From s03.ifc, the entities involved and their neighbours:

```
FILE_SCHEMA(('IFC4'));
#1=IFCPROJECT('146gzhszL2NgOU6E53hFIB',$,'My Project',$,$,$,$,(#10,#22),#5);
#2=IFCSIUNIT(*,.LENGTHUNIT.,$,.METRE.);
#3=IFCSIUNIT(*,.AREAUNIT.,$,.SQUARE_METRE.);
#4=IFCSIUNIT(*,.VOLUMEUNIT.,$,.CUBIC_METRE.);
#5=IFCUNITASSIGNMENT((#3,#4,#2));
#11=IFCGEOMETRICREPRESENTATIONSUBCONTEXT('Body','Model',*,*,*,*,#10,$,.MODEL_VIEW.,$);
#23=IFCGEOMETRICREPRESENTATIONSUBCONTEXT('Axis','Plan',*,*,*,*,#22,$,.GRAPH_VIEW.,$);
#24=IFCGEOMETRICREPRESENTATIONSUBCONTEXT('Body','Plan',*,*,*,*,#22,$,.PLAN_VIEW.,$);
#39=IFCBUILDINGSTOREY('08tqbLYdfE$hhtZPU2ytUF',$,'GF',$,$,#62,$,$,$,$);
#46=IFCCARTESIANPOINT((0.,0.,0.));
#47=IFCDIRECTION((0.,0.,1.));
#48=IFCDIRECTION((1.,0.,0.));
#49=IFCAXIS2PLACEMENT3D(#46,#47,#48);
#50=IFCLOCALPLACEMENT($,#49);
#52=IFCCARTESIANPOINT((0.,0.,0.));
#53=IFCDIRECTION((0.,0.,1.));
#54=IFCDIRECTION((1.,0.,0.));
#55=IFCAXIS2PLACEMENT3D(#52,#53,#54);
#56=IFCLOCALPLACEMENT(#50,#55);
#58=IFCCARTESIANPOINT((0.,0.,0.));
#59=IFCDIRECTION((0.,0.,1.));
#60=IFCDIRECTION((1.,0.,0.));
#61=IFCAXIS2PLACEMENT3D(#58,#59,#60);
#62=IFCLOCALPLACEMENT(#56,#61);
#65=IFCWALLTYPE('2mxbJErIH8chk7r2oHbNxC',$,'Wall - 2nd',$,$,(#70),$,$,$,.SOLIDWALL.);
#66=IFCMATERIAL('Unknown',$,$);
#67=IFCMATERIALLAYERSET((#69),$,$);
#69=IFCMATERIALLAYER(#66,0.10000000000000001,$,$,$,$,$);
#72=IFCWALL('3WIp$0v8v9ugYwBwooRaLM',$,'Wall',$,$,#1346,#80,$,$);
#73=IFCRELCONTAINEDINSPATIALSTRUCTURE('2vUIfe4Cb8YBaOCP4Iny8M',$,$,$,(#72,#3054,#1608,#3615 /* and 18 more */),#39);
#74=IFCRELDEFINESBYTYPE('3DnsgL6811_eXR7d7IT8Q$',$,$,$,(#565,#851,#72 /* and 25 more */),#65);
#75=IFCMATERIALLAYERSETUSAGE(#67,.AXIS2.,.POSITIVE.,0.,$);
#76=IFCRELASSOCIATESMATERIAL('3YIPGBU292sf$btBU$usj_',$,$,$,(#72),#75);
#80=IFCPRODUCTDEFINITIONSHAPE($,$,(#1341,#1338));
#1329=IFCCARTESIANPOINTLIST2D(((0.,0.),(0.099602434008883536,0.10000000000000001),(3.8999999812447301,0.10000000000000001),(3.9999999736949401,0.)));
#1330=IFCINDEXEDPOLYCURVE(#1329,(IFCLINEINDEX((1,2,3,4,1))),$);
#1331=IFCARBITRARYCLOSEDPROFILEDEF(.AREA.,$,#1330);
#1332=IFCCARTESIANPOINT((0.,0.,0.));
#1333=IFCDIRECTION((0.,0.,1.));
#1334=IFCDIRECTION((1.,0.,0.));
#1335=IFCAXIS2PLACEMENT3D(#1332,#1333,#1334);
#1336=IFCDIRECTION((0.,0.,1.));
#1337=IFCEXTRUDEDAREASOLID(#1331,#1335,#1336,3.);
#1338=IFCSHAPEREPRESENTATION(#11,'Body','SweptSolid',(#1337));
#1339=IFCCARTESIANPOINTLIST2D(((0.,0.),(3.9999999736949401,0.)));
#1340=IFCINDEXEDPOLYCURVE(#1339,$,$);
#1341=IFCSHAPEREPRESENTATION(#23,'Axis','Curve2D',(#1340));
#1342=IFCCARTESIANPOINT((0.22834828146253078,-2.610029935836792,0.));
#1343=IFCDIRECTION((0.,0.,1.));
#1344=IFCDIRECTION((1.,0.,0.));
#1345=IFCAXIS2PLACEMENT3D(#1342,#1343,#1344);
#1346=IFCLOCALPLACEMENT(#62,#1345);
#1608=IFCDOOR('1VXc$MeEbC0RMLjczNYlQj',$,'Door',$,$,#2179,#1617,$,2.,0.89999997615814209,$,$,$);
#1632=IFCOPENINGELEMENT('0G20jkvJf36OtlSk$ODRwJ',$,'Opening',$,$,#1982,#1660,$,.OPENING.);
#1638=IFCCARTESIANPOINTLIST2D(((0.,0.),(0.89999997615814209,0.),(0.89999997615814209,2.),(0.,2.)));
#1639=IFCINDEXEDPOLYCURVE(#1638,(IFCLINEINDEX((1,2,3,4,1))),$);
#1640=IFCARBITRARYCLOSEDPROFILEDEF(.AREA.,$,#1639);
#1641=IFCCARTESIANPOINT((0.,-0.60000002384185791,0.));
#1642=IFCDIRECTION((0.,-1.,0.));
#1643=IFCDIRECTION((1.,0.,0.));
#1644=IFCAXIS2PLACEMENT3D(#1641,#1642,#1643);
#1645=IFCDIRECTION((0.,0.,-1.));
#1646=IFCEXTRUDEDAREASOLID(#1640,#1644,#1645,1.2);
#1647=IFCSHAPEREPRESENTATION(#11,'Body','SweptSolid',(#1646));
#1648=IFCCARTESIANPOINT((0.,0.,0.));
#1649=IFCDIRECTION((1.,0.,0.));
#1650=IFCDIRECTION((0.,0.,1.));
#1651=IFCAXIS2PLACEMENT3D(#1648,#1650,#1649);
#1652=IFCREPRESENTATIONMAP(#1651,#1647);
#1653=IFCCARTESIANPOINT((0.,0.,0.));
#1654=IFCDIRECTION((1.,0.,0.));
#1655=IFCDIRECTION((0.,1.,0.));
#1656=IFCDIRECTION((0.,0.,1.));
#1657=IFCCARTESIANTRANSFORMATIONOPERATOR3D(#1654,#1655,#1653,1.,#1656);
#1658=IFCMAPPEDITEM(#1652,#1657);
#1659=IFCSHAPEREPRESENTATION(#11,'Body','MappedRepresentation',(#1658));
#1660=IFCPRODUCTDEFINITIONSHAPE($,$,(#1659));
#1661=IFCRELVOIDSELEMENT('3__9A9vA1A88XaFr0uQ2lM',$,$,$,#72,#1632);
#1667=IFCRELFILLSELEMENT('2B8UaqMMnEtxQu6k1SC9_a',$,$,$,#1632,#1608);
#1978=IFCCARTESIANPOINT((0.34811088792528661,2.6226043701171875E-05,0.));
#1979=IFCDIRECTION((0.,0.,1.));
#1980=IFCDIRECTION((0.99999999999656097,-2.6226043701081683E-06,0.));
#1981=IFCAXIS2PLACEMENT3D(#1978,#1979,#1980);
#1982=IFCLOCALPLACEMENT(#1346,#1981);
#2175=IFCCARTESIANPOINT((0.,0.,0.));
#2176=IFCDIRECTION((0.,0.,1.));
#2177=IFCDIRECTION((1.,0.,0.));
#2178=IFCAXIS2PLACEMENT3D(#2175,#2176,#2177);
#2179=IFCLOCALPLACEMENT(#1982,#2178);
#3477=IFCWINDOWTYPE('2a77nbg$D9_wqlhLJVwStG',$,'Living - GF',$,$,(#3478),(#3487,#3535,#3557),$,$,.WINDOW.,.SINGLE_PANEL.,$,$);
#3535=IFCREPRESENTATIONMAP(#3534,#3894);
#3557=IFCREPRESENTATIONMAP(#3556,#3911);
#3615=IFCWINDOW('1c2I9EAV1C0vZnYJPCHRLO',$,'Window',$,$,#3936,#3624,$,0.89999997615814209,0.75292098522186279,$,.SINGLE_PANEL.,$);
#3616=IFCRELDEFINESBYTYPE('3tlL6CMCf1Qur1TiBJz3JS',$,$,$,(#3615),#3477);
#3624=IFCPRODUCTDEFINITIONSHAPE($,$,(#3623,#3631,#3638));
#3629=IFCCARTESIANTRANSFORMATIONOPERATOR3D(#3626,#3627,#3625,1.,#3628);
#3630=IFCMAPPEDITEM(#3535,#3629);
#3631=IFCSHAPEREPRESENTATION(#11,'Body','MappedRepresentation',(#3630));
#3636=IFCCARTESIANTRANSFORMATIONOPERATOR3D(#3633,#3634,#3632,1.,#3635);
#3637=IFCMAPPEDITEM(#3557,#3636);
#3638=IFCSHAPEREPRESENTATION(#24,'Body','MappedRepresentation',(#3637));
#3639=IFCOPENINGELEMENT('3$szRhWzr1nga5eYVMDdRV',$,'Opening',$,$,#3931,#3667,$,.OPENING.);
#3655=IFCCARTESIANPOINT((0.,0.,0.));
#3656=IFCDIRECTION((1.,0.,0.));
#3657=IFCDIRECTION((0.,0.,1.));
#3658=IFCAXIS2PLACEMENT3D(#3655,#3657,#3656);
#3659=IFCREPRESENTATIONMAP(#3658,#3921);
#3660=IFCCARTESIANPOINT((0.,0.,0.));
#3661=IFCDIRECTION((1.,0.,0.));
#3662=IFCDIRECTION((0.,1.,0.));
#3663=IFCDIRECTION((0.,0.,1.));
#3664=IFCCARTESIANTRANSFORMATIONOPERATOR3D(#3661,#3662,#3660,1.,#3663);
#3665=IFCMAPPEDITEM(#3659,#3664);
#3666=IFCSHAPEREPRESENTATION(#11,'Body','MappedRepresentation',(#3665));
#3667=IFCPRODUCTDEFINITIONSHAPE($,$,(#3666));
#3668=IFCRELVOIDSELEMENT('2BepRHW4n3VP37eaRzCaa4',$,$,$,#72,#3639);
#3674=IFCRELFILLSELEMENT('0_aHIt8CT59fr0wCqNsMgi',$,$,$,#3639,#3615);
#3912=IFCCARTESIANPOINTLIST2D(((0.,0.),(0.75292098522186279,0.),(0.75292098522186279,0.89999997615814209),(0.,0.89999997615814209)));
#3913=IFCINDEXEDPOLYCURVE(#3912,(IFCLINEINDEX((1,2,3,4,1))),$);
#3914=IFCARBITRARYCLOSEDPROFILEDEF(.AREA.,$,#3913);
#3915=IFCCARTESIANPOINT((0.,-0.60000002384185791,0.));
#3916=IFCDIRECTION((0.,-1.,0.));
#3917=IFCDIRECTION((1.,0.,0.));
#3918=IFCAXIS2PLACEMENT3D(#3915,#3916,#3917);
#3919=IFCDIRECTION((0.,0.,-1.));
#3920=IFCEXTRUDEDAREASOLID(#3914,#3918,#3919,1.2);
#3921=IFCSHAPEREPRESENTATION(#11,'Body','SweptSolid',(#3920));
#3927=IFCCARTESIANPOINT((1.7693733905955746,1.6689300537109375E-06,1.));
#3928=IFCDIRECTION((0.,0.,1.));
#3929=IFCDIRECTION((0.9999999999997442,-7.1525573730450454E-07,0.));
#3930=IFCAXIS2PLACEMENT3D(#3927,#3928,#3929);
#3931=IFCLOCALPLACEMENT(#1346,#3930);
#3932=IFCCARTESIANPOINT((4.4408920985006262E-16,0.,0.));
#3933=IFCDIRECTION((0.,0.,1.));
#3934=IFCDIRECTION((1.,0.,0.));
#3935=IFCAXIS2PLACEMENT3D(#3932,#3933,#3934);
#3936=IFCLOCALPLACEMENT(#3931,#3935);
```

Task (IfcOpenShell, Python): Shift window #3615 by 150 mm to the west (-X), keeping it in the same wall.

```python
import ifcopenshell
import ifcopenshell.api.geometry
import ifcopenshell.util.placement

model = ifcopenshell.open("s03.ifc")

window = model.by_guid("1c2I9EAV1C0vZnYJPCHRLO")
opening = window.FillsVoids[0].RelatingOpeningElement
wall = opening.VoidsElements[0].RelatingBuildingElement

wall_matrix = ifcopenshell.util.placement.get_local_placement(wall.ObjectPlacement)
shift = wall_matrix[:3, 0] * -0.15
before = ifcopenshell.util.placement.get_local_placement(window.ObjectPlacement)[:3, 3].copy()

# The window is placed relative to its opening, so it follows when the opening moves.
matrix = ifcopenshell.util.placement.get_local_placement(opening.ObjectPlacement)
matrix[:3, 3] += shift
ifcopenshell.api.geometry.edit_object_placement(
    model, product=opening, matrix=matrix, is_si=False, should_transform_children=True
)

after = ifcopenshell.util.placement.get_local_placement(window.ObjectPlacement)[:3, 3]
print("window moved by", (after - before).round(3) + 0.0)

model.write("s03_rev.ifc")
```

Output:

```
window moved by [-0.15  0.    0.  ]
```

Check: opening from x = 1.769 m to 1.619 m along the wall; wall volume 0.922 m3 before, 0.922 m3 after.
